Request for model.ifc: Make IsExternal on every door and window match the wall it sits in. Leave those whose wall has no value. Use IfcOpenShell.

First a look at what the model holds.

```python
import ifcopenshell
import ifcopenshell.util.element

model = ifcopenshell.open("model.ifc")
print(model.schema)
seen = {}
for e in model.by_type("IfcDoor") + model.by_type("IfcWindow"):
    if not e.FillsVoids:
        continue
    host = e.FillsVoids[0].RelatingOpeningElement.VoidsElements[0].RelatingBuildingElement
    own = ifcopenshell.util.element.get_pset(e, f"Pset_{e.is_a()[3:].removesuffix('StandardCase')}Common", "IsExternal")
    wall = ifcopenshell.util.element.get_pset(host, "Pset_WallCommon", "IsExternal")
    seen[e.is_a(), own, wall] = seen.get((e.is_a(), own, wall), 0) + 1
for (cls, own, wall), count in sorted(seen.items(), key=str):
    print(count, cls, "IsExternal:", own, "| host wall:", wall)
```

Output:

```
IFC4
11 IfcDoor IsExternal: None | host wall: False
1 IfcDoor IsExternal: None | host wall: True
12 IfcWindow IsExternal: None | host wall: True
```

```python
import ifcopenshell
import ifcopenshell.api.pset
import ifcopenshell.util.element

model = ifcopenshell.open("model.ifc")

count = 0
for ifc_class, pset_name in (("IfcDoor", "Pset_DoorCommon"), ("IfcWindow", "Pset_WindowCommon")):
    for e in model.by_type(ifc_class):
        if not e.FillsVoids:
            continue
        host = e.FillsVoids[0].RelatingOpeningElement.VoidsElements[0].RelatingBuildingElement
        external = ifcopenshell.util.element.get_pset(host, "Pset_WallCommon", "IsExternal")
        if external is None or ifcopenshell.util.element.get_pset(e, pset_name, "IsExternal") == external:
            continue
        pset = ifcopenshell.api.pset.add_pset(model, product=e, name=pset_name)
        ifcopenshell.api.pset.edit_pset(model, pset=pset, properties={"IsExternal": external})
        count += 1

print(count, "updated")

model.write("model_rev.ifc")
```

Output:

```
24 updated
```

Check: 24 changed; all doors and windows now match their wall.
